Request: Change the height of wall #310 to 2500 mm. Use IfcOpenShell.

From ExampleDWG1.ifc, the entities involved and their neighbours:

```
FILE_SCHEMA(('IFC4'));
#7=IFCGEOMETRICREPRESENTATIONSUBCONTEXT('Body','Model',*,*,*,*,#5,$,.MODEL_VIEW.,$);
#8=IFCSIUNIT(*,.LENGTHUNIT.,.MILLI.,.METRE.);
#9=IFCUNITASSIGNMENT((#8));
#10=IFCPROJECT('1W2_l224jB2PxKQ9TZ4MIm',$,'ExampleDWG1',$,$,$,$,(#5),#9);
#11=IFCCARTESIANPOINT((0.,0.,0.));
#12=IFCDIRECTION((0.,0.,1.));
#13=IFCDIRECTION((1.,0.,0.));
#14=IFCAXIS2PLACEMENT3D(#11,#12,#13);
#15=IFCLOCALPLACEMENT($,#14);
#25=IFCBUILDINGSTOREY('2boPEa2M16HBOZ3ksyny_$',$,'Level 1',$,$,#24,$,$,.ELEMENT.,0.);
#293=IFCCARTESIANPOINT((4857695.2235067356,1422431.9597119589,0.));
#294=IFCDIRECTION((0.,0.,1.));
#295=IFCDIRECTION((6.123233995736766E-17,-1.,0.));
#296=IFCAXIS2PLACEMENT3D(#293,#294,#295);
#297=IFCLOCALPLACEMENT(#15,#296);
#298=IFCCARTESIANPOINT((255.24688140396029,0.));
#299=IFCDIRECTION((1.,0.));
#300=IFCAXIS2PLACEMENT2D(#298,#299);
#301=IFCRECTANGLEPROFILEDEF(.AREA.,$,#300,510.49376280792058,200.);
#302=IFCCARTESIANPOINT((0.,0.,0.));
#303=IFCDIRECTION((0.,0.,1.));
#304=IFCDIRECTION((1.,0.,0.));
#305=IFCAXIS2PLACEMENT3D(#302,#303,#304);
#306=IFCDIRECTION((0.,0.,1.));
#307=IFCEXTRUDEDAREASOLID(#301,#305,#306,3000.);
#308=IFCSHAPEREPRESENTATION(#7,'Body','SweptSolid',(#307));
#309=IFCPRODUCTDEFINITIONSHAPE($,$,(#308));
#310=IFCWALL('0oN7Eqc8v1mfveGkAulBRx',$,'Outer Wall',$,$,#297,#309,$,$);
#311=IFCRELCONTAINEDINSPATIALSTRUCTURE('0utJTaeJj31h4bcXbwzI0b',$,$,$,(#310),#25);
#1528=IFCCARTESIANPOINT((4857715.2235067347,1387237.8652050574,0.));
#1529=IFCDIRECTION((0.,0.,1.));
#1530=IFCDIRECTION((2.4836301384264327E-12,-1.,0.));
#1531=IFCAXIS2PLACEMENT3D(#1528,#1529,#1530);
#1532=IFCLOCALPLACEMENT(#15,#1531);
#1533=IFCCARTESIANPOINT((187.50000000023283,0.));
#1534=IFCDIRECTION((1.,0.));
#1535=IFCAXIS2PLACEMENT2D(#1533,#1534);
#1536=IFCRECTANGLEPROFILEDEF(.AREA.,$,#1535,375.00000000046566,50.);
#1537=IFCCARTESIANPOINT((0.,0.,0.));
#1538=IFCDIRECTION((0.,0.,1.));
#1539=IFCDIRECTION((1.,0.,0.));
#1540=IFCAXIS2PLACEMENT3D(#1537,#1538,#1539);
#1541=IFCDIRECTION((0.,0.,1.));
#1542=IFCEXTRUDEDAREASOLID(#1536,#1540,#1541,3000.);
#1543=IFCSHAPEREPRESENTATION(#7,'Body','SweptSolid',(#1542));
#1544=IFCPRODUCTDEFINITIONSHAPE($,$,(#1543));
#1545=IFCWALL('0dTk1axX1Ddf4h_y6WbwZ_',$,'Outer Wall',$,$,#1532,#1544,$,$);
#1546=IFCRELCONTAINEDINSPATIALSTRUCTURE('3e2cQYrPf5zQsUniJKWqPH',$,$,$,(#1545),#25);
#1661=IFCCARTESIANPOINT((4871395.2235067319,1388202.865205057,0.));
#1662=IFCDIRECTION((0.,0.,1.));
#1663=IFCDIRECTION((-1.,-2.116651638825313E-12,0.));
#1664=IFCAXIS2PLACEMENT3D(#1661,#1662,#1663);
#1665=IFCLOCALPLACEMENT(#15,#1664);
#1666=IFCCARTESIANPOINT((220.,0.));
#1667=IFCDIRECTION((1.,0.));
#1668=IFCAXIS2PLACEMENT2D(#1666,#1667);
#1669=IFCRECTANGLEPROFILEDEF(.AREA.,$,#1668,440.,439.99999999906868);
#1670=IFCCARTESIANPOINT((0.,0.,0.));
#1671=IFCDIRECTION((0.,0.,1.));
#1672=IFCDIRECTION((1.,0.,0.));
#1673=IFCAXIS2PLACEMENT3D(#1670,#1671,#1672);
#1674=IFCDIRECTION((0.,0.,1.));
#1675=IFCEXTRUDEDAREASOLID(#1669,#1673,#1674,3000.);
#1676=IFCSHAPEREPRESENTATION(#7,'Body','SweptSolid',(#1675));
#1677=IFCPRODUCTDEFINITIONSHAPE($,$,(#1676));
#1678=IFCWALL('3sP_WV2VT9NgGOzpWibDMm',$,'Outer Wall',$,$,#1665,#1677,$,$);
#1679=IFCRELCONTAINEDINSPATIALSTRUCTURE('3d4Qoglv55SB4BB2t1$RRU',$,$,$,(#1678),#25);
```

```python
import ifcopenshell
import ifcopenshell.geom
import ifcopenshell.util.representation
import ifcopenshell.util.shape
import ifcopenshell.util.unit

model = ifcopenshell.open("ExampleDWG1.ifc")
unit_scale = ifcopenshell.util.unit.calculate_unit_scale(model)
settings = ifcopenshell.geom.settings()


def volume(element):
    """Net volume in cubic metres, openings subtracted."""
    shape = ifcopenshell.geom.create_shape(settings, element)
    return ifcopenshell.util.shape.get_volume(shape.geometry)


wall = model.by_guid("0oN7Eqc8v1mfveGkAulBRx")
before = volume(wall)

body = ifcopenshell.util.representation.get_representation(wall, "Model", "Body")
solid = body.Items[0]
old_height = solid.Depth
solid.Depth = 2.5 / unit_scale
after = volume(wall)

print(f"height {old_height:g} -> {solid.Depth:g}, volume {before:.3f} -> {after:.3f} m3")

model.write("ExampleDWG1-out.ifc")
```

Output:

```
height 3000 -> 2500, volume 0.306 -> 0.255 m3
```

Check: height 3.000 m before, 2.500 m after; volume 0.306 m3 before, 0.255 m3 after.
